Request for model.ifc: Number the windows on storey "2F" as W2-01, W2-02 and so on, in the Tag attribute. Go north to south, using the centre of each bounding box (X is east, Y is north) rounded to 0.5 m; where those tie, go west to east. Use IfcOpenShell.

First a look at what the model holds.

```python
import ifcopenshell
import ifcopenshell.util.element
import ifcopenshell.util.placement

model = ifcopenshell.open("model.ifc")
print(model.schema)
storey = next(s for s in model.by_type("IfcBuildingStorey") if s.Name == "2F")
windows = [e for e in ifcopenshell.util.element.get_decomposition(storey) if e.is_a("IfcWindow")]
for e in sorted(windows, key=lambda e: e.id()):
    origin = ifcopenshell.util.placement.get_local_placement(e.ObjectPlacement)[:3, 3]
    print(e.id(), e.Tag, e.Name, origin.round(2) + 0.0, sep=" | ")
```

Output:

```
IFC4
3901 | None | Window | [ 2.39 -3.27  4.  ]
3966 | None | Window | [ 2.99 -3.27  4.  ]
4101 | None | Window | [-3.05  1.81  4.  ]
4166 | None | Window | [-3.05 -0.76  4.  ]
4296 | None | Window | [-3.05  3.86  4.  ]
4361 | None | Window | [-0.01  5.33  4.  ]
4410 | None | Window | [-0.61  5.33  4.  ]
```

```python
import ifcopenshell
import ifcopenshell.geom
import ifcopenshell.util.element
import ifcopenshell.util.shape

model = ifcopenshell.open("model.ifc")
settings = ifcopenshell.geom.settings()
settings.set("use-world-coords", True)


def centre(element):
    shape = ifcopenshell.geom.create_shape(settings, element)
    return ifcopenshell.util.shape.get_bbox_centroid(shape.geometry)


storey = next(s for s in model.by_type("IfcBuildingStorey") if s.Name == "2F")
windows = [e for e in ifcopenshell.util.element.get_decomposition(storey) if e.is_a("IfcWindow")]

# Insertion points can sit at a corner or the storey origin, so sort by the geometry (in metres).
centres = {e: centre(e) for e in windows}
windows.sort(key=lambda e: (-round(centres[e][1] / 0.5), centres[e][0]))

for i, e in enumerate(windows, start=1):
    number = f"W2-{i:02d}"
    e.Tag = number
    print(e.id(), number)

model.write("model_updated.ifc")
```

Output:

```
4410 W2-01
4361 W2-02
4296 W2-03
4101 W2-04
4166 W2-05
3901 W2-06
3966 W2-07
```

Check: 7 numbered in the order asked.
